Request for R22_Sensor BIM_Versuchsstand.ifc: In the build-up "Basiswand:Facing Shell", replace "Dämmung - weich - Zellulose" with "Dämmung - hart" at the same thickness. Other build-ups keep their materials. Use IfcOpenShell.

First a look at what the model holds.

```python
import ifcopenshell
import ifcopenshell.util.element

model = ifcopenshell.open("R22_Sensor BIM_Versuchsstand.ifc")
print(model.schema)
for layer_set in model.by_type("IfcMaterialLayerSet"):
    if layer_set.LayerSetName == "Basiswand:Facing Shell":
        for layer in layer_set.MaterialLayers:
            print(layer.id(), layer.Material and layer.Material.Name, layer.LayerThickness, sep=" | ")
        print(len(ifcopenshell.util.element.get_elements_by_material(model, layer_set)), "elements and types use it")
print(sorted(m.Name for m in model.by_type("IfcMaterial") if m.Name)[:60])
```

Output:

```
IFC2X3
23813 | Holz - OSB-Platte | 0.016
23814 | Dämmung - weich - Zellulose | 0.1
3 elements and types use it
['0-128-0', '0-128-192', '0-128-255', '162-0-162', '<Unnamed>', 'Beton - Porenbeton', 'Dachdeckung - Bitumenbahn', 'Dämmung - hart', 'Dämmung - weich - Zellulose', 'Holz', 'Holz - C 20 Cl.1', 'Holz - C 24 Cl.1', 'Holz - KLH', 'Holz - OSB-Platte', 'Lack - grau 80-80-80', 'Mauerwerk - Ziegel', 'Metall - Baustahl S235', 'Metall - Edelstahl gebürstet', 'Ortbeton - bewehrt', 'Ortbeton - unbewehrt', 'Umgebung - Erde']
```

```python
import ifcopenshell
import ifcopenshell.api.material

model = ifcopenshell.open("R22_Sensor BIM_Versuchsstand.ifc")

layer_set = next(s for s in model.by_type("IfcMaterialLayerSet") if s.LayerSetName == "Basiswand:Facing Shell")
layer = next(l for l in layer_set.MaterialLayers if l.Material and l.Material.Name == "Dämmung - weich - Zellulose")
material = next(m for m in model.by_type("IfcMaterial") if m.Name == "Dämmung - hart")

# Point this one layer at the other material; renaming the old one would change it everywhere.
ifcopenshell.api.material.edit_layer(model, layer=layer, attributes={}, material=material)

print([l.Material.Name if l.Material else None for l in layer_set.MaterialLayers])

model.write("R22_Sensor BIM_Versuchsstand_updated.ifc")
```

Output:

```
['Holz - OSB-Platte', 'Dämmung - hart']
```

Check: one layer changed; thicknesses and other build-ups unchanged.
